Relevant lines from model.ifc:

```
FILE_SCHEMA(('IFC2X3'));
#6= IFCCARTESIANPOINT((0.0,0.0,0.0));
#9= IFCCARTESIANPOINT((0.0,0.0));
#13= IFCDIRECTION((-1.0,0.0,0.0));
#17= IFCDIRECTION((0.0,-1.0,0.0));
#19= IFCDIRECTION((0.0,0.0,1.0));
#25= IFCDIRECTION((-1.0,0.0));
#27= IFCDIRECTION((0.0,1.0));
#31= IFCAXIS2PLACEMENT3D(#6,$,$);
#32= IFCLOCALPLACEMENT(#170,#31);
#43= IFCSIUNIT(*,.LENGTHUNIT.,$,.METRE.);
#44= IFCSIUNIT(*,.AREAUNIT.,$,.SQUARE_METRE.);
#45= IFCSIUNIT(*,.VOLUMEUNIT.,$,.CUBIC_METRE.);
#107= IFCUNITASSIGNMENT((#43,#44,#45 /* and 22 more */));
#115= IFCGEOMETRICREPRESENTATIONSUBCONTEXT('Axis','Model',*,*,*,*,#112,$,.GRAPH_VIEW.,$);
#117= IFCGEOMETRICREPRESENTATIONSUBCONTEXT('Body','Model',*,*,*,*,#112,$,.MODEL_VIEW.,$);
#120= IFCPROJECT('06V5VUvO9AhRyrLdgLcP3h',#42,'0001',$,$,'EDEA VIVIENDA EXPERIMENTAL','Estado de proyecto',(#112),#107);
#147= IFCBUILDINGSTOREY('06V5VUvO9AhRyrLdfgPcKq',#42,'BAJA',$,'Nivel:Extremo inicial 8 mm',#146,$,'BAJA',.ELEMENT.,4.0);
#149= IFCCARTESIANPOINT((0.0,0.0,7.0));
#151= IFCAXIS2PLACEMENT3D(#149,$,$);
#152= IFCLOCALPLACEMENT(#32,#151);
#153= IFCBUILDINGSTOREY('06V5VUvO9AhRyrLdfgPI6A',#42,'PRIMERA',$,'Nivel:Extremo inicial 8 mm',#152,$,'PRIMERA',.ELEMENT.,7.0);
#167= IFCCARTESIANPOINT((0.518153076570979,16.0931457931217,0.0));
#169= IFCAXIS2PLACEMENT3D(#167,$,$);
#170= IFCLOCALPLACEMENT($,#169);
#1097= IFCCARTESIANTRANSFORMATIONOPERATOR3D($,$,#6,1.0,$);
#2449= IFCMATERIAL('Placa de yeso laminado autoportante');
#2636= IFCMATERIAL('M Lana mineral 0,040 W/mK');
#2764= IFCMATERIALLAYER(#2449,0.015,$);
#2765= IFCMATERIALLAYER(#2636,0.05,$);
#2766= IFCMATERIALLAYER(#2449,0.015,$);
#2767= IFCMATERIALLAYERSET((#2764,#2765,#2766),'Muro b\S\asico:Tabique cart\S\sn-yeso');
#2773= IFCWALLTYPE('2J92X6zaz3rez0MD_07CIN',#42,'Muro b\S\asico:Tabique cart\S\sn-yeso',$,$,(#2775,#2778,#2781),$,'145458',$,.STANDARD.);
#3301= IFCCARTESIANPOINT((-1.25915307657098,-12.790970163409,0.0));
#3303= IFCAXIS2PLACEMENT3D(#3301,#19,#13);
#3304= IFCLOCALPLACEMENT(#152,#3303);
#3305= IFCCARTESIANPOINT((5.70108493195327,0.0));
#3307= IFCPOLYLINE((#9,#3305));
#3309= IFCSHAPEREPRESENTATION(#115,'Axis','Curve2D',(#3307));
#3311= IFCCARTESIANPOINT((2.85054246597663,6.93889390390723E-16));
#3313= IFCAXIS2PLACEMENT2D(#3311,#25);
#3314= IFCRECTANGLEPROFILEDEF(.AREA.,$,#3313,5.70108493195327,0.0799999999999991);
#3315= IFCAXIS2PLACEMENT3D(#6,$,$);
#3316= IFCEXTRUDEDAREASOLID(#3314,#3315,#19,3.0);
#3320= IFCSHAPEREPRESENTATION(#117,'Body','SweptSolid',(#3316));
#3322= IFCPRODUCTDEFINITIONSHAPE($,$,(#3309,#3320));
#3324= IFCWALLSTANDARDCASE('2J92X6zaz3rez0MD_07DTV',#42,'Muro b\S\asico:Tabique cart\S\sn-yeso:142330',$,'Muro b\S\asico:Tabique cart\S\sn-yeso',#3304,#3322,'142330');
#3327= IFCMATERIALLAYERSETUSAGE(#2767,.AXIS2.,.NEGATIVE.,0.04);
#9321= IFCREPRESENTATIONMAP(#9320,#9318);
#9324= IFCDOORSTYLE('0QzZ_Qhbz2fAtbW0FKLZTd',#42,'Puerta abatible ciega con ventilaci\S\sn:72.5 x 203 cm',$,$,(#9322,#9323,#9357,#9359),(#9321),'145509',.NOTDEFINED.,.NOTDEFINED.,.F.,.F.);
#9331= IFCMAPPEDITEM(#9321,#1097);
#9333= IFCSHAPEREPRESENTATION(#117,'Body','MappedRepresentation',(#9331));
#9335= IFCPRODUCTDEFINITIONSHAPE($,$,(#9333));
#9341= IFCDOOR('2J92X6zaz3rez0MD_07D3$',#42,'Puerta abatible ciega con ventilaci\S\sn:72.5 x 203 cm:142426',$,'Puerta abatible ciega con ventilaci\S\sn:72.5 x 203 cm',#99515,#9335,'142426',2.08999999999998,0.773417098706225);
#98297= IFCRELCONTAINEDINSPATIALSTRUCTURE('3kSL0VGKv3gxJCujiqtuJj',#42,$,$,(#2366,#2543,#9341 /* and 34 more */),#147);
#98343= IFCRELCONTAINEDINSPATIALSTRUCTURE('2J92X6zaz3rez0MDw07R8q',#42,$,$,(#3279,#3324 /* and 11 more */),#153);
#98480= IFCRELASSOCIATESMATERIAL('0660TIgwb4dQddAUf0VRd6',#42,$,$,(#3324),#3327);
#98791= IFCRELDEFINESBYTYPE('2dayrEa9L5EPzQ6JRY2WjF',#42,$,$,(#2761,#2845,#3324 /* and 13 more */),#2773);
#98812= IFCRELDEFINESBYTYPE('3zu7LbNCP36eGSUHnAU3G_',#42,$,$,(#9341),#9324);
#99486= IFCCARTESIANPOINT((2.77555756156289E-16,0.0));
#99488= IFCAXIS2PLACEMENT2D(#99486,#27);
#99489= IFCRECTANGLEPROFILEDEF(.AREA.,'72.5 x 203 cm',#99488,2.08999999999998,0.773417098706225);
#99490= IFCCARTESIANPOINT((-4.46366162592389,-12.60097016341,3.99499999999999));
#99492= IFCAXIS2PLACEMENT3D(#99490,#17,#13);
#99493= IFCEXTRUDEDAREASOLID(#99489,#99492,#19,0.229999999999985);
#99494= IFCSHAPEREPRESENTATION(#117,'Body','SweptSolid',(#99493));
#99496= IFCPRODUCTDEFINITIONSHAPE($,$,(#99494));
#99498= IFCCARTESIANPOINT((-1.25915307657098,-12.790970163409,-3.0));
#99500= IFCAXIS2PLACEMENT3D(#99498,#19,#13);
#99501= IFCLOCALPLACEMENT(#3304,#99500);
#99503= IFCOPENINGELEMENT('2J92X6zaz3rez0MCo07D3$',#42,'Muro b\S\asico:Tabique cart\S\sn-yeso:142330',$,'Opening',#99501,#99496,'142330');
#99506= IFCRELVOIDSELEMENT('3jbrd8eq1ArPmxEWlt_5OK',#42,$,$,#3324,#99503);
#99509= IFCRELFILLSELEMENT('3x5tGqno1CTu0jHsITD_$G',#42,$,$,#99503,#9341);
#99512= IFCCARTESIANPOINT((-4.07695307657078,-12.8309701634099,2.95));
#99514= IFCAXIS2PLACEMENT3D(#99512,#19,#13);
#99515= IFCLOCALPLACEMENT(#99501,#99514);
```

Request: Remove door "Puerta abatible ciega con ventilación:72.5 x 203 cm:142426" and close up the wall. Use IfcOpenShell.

```python
import ifcopenshell
import ifcopenshell.api.feature
import ifcopenshell.api.root
import ifcopenshell.geom
import ifcopenshell.util.shape

model = ifcopenshell.open("model.ifc")
settings = ifcopenshell.geom.settings()


def volume(element):
    """Net volume in cubic metres, openings subtracted."""
    shape = ifcopenshell.geom.create_shape(settings, element)
    return ifcopenshell.util.shape.get_volume(shape.geometry)


door = model.by_id(9341)
opening = door.FillsVoids[0].RelatingOpeningElement
wall = opening.VoidsElements[0].RelatingBuildingElement
before = volume(wall)

ifcopenshell.api.root.remove_product(model, product=door)
ifcopenshell.api.feature.remove_feature(model, feature=opening)

after = volume(wall)

print(f"wall volume {before:.3f} -> {after:.3f} m3")

model.write("model_updated.ifc")
```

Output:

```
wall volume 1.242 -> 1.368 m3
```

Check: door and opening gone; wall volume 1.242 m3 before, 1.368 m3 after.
